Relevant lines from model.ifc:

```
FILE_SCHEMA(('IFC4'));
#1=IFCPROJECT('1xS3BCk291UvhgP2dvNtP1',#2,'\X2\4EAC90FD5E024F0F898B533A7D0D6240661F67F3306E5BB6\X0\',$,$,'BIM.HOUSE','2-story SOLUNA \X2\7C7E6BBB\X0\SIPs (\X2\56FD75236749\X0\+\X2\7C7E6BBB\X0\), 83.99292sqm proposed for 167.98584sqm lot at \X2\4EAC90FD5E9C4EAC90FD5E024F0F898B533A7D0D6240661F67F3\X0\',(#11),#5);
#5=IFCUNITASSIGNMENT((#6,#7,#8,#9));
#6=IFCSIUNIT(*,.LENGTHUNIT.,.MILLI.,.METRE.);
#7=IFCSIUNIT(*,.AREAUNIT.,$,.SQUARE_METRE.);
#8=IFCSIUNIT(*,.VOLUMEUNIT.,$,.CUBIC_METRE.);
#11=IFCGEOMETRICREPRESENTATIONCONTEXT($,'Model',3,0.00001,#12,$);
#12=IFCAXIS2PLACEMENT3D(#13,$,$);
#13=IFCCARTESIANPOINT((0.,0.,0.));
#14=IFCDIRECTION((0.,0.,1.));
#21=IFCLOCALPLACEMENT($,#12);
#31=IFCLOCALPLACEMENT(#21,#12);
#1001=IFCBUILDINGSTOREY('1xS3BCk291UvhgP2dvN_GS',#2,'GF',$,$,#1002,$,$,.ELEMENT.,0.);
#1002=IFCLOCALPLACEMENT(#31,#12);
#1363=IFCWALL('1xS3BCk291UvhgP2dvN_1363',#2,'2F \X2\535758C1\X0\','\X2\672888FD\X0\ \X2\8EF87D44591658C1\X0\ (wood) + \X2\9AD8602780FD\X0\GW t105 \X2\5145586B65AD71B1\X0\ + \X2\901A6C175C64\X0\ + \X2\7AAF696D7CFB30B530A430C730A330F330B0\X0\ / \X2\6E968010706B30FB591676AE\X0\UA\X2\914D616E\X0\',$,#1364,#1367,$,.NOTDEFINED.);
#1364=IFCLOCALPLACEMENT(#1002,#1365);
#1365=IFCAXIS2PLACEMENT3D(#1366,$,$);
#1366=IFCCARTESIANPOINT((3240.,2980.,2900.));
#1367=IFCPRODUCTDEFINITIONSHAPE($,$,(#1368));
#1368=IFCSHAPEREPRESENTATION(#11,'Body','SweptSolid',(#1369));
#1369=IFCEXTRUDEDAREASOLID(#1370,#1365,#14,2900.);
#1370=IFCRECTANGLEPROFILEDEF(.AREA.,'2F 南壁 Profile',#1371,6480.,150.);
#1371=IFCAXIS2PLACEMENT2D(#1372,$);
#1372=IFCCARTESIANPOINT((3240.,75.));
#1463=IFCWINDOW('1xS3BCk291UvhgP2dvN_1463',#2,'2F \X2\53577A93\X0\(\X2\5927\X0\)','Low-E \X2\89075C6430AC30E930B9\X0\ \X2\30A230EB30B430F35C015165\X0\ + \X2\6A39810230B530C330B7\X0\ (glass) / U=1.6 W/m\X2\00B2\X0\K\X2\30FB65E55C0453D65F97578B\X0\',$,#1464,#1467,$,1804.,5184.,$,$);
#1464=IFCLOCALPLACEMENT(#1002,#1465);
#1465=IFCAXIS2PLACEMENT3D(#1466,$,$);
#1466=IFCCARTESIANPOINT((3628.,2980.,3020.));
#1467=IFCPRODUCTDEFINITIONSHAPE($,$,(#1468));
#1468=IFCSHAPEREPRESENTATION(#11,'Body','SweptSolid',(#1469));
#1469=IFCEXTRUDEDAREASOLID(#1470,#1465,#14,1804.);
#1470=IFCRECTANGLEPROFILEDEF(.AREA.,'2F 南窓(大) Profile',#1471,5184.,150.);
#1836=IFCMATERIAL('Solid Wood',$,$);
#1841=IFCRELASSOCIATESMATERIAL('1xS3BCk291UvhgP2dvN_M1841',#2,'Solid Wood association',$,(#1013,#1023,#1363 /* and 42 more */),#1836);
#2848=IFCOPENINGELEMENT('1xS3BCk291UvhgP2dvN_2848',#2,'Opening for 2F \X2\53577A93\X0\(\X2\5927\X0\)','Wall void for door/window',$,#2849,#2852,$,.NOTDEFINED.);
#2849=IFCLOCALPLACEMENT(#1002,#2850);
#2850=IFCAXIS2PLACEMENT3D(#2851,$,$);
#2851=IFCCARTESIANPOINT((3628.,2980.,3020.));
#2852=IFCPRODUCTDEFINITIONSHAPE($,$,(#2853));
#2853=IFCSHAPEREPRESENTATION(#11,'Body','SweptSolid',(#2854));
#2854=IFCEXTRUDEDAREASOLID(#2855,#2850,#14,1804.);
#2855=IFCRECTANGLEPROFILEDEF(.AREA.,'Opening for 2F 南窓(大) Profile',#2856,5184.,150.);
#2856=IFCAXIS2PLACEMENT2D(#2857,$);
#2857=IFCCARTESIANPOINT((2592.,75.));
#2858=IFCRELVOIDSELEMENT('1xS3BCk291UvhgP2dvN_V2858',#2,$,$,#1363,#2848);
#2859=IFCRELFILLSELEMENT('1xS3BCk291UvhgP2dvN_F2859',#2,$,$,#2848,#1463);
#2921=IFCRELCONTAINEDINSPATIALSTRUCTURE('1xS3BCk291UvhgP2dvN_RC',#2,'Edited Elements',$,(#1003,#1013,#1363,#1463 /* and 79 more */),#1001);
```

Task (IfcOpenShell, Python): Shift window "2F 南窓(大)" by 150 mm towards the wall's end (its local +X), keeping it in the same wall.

```python
import ifcopenshell
import ifcopenshell.api.geometry
import ifcopenshell.util.placement
import ifcopenshell.util.unit

model = ifcopenshell.open("model.ifc")
unit_scale = ifcopenshell.util.unit.calculate_unit_scale(model)

window = model.by_id(1463)
opening = window.FillsVoids[0].RelatingOpeningElement
wall = opening.VoidsElements[0].RelatingBuildingElement

wall_matrix = ifcopenshell.util.placement.get_local_placement(wall.ObjectPlacement)
shift = wall_matrix[:3, 0] * 0.15 / unit_scale
before = ifcopenshell.util.placement.get_local_placement(window.ObjectPlacement)[:3, 3].copy()

# The window is not placed relative to its opening, so move both.
for product in (opening, window):
    matrix = ifcopenshell.util.placement.get_local_placement(product.ObjectPlacement)
    matrix[:3, 3] += shift
    ifcopenshell.api.geometry.edit_object_placement(model, product=product, matrix=matrix, is_si=False)

after = ifcopenshell.util.placement.get_local_placement(window.ObjectPlacement)[:3, 3]
print("window moved by", (after - before).round(3) + 0.0)

model.write("model-out.ifc")
```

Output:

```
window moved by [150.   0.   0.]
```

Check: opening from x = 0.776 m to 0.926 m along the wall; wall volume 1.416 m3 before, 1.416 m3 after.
